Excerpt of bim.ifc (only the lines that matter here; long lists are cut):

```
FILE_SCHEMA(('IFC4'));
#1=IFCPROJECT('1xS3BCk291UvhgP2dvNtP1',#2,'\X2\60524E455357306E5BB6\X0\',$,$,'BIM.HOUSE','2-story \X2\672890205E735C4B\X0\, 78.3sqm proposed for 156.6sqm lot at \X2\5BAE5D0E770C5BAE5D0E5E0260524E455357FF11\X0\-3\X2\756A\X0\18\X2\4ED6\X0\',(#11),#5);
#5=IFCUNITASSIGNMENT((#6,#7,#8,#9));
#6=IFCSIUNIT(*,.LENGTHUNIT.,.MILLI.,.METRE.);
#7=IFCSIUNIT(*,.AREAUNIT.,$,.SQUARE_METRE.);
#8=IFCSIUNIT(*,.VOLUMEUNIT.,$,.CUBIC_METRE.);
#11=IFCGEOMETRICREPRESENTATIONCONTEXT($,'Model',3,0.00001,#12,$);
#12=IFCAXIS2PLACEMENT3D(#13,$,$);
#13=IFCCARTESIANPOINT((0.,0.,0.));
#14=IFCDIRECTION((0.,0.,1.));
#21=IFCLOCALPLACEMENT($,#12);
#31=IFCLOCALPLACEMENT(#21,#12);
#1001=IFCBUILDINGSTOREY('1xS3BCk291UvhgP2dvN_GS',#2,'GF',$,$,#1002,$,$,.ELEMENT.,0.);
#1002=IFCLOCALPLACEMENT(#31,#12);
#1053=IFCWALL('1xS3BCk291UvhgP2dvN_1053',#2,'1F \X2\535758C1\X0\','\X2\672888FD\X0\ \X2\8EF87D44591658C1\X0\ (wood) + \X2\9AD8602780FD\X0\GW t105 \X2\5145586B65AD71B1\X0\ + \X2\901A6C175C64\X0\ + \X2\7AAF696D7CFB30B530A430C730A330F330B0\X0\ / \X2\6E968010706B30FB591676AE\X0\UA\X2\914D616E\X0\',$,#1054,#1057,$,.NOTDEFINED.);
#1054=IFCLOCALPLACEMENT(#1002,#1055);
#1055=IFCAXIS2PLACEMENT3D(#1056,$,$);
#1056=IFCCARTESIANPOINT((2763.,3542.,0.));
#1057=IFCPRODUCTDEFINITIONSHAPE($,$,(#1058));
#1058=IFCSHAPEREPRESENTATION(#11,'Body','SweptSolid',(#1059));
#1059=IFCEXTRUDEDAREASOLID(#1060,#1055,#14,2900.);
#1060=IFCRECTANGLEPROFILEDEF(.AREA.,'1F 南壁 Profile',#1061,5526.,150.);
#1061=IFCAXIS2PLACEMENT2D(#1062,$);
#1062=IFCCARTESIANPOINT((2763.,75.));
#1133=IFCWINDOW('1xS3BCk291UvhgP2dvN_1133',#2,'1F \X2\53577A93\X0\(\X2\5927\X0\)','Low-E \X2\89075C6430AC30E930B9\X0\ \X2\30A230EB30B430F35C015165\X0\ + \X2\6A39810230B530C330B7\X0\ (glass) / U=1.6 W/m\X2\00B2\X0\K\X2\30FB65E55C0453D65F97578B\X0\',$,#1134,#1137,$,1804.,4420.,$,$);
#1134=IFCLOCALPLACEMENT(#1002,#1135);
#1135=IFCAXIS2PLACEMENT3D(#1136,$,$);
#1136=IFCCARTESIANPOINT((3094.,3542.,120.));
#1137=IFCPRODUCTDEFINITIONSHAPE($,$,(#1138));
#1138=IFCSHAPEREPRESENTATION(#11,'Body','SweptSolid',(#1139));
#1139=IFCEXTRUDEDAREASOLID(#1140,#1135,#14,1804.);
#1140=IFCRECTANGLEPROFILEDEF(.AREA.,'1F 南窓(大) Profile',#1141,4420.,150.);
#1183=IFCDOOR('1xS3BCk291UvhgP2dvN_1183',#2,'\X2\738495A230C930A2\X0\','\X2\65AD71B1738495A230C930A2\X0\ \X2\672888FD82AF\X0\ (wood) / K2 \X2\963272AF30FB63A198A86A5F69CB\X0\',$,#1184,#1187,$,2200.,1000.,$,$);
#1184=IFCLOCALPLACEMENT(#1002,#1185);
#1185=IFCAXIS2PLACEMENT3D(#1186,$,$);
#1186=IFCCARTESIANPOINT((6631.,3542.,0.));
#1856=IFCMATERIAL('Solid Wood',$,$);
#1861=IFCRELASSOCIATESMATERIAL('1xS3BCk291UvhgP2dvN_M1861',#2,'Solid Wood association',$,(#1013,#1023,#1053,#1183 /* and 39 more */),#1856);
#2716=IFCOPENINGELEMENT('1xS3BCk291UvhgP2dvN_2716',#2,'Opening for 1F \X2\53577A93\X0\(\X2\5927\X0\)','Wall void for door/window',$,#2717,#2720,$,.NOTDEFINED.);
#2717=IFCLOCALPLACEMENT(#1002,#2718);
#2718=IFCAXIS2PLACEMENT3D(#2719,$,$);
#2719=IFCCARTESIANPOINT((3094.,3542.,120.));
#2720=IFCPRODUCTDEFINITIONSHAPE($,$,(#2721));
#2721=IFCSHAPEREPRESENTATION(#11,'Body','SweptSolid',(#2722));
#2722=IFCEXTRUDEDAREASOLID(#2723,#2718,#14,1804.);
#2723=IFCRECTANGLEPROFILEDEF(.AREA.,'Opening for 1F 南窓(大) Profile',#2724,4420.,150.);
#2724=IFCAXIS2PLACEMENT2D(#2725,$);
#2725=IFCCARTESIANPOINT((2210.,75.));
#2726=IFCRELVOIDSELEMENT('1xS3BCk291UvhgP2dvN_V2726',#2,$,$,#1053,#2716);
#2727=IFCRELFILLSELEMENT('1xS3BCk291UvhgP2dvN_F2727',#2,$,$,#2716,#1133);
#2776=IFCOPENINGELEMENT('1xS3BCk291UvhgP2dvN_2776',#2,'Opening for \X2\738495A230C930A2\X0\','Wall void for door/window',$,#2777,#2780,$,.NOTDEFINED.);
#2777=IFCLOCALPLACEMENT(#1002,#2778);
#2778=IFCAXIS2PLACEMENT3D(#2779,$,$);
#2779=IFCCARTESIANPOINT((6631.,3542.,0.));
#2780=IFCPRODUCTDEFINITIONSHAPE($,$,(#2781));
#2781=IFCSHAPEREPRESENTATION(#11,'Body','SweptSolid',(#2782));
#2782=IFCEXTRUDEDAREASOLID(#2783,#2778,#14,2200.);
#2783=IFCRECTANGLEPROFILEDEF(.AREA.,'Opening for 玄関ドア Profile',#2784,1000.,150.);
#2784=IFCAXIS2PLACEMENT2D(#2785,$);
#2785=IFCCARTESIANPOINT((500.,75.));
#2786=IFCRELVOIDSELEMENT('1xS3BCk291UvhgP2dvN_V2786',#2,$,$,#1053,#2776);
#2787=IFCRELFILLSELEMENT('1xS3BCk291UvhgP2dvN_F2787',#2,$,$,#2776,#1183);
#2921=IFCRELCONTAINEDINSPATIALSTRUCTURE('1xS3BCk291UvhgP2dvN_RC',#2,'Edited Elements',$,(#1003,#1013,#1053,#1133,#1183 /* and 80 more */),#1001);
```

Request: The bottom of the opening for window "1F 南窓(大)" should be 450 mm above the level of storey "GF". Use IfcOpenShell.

```python
import numpy as np
import ifcopenshell
import ifcopenshell.api.geometry
import ifcopenshell.geom
import ifcopenshell.util.element
import ifcopenshell.util.placement
import ifcopenshell.util.shape
import ifcopenshell.util.unit

model = ifcopenshell.open("bim.ifc")
unit_scale = ifcopenshell.util.unit.calculate_unit_scale(model)

window = model.by_guid("1xS3BCk291UvhgP2dvN_1133")
opening = window.FillsVoids[0].RelatingOpeningElement
storey = ifcopenshell.util.element.get_container(window, ifc_class="IfcBuildingStorey")
level = ifcopenshell.util.placement.get_local_placement(storey.ObjectPlacement)[2, 3]

# The opening's origin need not be at the sill, so measure its lowest point.
shape = ifcopenshell.geom.create_shape(ifcopenshell.geom.settings(), opening)
bottom = ifcopenshell.util.shape.get_shape_bottom_elevation(shape, shape.geometry) / unit_scale
dz = level + 450.0 - bottom

shift = np.array([0.0, 0.0, dz])
# The window is not placed relative to its opening, so move both.
for product in (opening, window):
    matrix = ifcopenshell.util.placement.get_local_placement(product.ObjectPlacement)
    matrix[:3, 3] += shift
    ifcopenshell.api.geometry.edit_object_placement(model, product=product, matrix=matrix, is_si=False)

print(f"moved by {dz * unit_scale:+.3f} m")

model.write("bim_updated.ifc")
```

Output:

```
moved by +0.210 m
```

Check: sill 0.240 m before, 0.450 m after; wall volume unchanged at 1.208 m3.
